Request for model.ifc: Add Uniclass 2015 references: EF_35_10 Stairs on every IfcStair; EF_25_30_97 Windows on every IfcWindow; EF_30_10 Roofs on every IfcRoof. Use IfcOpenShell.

First a look at what the model holds.

```python
import ifcopenshell

model = ifcopenshell.open("model.ifc")
print(model.schema)
print("classifications:", [c.Name for c in model.by_type("IfcClassification")])
for ifc_class in ("IfcDoor", "IfcRoof", "IfcStair", "IfcWall", "IfcWindow"):
    print(ifc_class, len(model.by_type(ifc_class)))
```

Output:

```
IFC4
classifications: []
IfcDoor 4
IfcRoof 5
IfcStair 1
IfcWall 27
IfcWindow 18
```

```python
import ifcopenshell
import ifcopenshell.api.classification

model = ifcopenshell.open("model.ifc")

system = ifcopenshell.api.classification.add_classification(model, classification="Uniclass 2015")

codes = {
    "IfcStair": ("EF_35_10", "Stairs"),
    "IfcWindow": ("EF_25_30_97", "Windows"),
    "IfcRoof": ("EF_30_10", "Roofs"),
}
for ifc_class, (code, name) in codes.items():
    products = model.by_type(ifc_class)
    ifcopenshell.api.classification.add_reference(
        model, products=products, classification=system, identification=code, name=name
    )
    print(code, len(products))

model.write("model_rev.ifc")
```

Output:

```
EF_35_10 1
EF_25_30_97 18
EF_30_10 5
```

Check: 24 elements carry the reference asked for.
